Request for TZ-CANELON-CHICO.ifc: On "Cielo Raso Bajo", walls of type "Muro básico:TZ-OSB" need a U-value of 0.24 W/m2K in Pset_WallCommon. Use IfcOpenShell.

First a look at what the model holds.

```python
import ifcopenshell
import ifcopenshell.util.element

model = ifcopenshell.open("TZ-CANELON-CHICO.ifc")
print(model.schema)
storey = next(s for s in model.by_type("IfcBuildingStorey") if s.Name == "Cielo Raso Bajo")
walls = [e for e in ifcopenshell.util.element.get_decomposition(storey) if e.is_a("IfcWall")]
seen = {}
for e in walls:
    element_type = ifcopenshell.util.element.get_type(e)
    key = (element_type.Name if element_type != e and element_type else None, ifcopenshell.util.element.get_pset(e, "Pset_WallCommon", "ThermalTransmittance"))
    seen[key] = seen.get(key, 0) + 1
for (name, value), count in sorted(seen.items(), key=str):
    print(count, "x", name, "|", value)
```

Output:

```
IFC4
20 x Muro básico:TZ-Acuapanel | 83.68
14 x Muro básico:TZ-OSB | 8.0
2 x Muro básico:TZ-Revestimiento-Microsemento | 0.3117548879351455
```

```python
import ifcopenshell
import ifcopenshell.api.pset
import ifcopenshell.util.element

model = ifcopenshell.open("TZ-CANELON-CHICO.ifc")

storey = next(s for s in model.by_type("IfcBuildingStorey") if s.Name == "Cielo Raso Bajo")
walls = [e for e in ifcopenshell.util.element.get_decomposition(storey) if e.is_a("IfcWall")]

count = 0
for e in walls:
    element_type = ifcopenshell.util.element.get_type(e)
    if element_type in (None, e) or element_type.Name != "Muro básico:TZ-OSB":
        continue
    # add_pset returns the element's existing set when there is one.
    pset = ifcopenshell.api.pset.add_pset(model, product=e, name="Pset_WallCommon")
    ifcopenshell.api.pset.edit_pset(model, pset=pset, properties={"ThermalTransmittance": 0.24})
    count += 1

print(count, "walls updated")

model.write("TZ-CANELON-CHICO_rev.ifc")
```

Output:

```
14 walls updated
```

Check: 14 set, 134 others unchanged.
